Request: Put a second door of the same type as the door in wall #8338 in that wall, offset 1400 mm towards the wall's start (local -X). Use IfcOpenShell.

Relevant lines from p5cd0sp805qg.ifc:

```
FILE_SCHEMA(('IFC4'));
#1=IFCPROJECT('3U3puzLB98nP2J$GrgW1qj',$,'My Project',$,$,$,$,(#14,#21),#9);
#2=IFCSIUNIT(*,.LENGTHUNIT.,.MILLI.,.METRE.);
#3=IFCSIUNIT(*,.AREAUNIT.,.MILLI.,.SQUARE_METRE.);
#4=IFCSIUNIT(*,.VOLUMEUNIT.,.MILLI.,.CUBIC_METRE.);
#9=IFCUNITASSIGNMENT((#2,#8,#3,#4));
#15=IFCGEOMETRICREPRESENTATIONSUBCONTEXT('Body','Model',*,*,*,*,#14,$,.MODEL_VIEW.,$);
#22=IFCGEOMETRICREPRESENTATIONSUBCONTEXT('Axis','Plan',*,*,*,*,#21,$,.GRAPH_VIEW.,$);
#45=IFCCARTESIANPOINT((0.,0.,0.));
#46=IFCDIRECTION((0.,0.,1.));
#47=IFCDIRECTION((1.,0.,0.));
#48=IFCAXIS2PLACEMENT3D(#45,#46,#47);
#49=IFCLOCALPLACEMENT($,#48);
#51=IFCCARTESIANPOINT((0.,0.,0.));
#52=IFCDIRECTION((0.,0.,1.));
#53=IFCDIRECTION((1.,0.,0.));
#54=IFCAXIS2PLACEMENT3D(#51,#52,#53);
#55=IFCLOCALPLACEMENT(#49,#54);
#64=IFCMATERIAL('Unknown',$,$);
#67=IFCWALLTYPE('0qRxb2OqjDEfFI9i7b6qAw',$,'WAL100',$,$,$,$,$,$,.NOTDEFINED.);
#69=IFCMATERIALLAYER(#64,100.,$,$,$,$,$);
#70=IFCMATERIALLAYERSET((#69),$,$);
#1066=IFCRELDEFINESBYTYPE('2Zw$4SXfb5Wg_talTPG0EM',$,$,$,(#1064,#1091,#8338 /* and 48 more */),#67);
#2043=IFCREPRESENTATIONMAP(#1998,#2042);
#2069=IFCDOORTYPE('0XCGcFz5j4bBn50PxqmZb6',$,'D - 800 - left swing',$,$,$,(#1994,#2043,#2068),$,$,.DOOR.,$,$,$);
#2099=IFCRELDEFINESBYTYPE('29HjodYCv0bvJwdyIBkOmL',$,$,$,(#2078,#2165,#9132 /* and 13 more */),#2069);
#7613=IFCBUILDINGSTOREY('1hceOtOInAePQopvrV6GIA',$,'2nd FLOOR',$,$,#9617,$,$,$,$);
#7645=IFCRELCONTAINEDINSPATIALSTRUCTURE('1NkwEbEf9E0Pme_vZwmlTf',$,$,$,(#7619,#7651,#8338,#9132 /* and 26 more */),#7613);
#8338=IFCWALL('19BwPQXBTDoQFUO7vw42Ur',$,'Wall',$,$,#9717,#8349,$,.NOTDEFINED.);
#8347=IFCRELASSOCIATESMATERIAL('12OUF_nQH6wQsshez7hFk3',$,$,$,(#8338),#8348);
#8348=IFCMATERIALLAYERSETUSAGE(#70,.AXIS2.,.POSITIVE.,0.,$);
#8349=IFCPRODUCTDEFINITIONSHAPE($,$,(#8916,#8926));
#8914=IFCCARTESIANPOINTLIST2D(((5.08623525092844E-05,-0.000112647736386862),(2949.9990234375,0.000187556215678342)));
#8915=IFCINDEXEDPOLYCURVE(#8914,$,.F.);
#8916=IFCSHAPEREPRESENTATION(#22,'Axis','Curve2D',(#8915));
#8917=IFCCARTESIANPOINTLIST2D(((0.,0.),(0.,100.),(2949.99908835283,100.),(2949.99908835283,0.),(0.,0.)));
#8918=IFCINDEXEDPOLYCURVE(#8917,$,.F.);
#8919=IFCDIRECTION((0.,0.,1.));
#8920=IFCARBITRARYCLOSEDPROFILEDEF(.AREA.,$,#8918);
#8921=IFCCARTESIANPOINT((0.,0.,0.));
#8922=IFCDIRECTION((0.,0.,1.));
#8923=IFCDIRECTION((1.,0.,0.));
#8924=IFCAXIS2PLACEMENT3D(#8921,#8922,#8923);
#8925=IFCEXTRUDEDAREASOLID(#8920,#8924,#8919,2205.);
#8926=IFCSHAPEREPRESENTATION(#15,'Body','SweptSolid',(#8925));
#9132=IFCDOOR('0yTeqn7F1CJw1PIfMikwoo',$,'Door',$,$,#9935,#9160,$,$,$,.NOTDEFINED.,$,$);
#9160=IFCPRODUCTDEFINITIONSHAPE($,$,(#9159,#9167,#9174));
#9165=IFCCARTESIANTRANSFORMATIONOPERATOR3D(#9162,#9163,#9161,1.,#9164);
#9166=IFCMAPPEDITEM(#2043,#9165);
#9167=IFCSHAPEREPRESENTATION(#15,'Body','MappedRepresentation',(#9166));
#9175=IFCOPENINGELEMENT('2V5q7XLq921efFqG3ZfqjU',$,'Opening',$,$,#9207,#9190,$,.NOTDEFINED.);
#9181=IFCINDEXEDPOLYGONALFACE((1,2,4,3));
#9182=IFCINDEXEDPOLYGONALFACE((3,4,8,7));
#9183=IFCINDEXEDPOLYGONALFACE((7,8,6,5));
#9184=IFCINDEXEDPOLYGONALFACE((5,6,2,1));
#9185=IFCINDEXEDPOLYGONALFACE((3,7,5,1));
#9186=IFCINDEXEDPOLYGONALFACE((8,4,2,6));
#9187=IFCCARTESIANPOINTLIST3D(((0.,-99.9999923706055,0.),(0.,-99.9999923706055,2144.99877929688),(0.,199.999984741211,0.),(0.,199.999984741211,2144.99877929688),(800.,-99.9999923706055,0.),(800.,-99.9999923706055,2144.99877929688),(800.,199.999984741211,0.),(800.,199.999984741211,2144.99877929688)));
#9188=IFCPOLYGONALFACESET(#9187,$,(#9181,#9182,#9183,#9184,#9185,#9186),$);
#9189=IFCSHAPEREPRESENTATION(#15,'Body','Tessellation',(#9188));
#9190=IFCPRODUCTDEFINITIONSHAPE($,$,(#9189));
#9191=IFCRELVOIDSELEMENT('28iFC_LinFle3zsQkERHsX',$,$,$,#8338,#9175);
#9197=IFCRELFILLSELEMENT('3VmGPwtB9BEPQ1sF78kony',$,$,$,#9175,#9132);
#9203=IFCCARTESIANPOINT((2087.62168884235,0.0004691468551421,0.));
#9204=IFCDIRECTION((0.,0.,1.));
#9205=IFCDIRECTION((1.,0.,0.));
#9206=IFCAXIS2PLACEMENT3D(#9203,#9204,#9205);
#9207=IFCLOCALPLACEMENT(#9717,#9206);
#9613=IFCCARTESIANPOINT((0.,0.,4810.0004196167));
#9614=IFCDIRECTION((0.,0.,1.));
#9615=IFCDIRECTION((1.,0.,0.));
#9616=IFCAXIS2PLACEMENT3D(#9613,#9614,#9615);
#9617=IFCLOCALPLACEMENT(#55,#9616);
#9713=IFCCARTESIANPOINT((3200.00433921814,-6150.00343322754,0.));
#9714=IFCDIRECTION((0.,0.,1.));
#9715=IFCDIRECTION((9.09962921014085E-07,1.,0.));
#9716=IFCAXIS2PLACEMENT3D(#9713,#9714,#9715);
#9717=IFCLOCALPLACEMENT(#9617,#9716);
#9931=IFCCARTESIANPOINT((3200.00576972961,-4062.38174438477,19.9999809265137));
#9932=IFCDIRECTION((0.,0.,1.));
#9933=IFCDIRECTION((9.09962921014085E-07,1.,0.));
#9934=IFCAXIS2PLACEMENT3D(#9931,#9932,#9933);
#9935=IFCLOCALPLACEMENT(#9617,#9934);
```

```python
import ifcopenshell
import ifcopenshell.api.feature
import ifcopenshell.api.geometry
import ifcopenshell.api.root
import ifcopenshell.geom
import ifcopenshell.util.element
import ifcopenshell.util.placement
import ifcopenshell.util.shape
import ifcopenshell.util.unit

model = ifcopenshell.open("p5cd0sp805qg.ifc")
unit_scale = ifcopenshell.util.unit.calculate_unit_scale(model)
settings = ifcopenshell.geom.settings()


def volume(element):
    """Net volume in cubic metres, openings subtracted."""
    shape = ifcopenshell.geom.create_shape(settings, element)
    return ifcopenshell.util.shape.get_volume(shape.geometry)


door = model.by_guid("0yTeqn7F1CJw1PIfMikwoo")
opening = door.FillsVoids[0].RelatingOpeningElement
wall = opening.VoidsElements[0].RelatingBuildingElement
before = volume(wall)
shift = ifcopenshell.util.placement.get_local_placement(wall.ObjectPlacement)[:3, 0] * -1.4 / unit_scale

# copy_class copies the void relationship, type, container and properties, but no geometry.
new_opening = ifcopenshell.api.root.copy_class(model, product=opening)
new_opening.Representation = ifcopenshell.util.element.copy_deep(
    model, opening.Representation, exclude=["IfcGeometricRepresentationContext", "IfcRepresentationMap"]
)
new_door = ifcopenshell.api.root.copy_class(model, product=door)
new_door.Representation = ifcopenshell.util.element.copy_deep(
    model, door.Representation, exclude=["IfcGeometricRepresentationContext", "IfcRepresentationMap"]
)
ifcopenshell.api.feature.add_filling(model, opening=new_opening, element=new_door)

for old, new in ((opening, new_opening), (door, new_door)):
    matrix = ifcopenshell.util.placement.get_local_placement(old.ObjectPlacement)
    matrix[:3, 3] += shift
    ifcopenshell.api.geometry.edit_object_placement(model, product=new, matrix=matrix, is_si=False)

after = volume(wall)

print(f"wall volume {before:.3f} -> {after:.3f} m3")

model.write("p5cd0sp805qg_updated.ifc")
```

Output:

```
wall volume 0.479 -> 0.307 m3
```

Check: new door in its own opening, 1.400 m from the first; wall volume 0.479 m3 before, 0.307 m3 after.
